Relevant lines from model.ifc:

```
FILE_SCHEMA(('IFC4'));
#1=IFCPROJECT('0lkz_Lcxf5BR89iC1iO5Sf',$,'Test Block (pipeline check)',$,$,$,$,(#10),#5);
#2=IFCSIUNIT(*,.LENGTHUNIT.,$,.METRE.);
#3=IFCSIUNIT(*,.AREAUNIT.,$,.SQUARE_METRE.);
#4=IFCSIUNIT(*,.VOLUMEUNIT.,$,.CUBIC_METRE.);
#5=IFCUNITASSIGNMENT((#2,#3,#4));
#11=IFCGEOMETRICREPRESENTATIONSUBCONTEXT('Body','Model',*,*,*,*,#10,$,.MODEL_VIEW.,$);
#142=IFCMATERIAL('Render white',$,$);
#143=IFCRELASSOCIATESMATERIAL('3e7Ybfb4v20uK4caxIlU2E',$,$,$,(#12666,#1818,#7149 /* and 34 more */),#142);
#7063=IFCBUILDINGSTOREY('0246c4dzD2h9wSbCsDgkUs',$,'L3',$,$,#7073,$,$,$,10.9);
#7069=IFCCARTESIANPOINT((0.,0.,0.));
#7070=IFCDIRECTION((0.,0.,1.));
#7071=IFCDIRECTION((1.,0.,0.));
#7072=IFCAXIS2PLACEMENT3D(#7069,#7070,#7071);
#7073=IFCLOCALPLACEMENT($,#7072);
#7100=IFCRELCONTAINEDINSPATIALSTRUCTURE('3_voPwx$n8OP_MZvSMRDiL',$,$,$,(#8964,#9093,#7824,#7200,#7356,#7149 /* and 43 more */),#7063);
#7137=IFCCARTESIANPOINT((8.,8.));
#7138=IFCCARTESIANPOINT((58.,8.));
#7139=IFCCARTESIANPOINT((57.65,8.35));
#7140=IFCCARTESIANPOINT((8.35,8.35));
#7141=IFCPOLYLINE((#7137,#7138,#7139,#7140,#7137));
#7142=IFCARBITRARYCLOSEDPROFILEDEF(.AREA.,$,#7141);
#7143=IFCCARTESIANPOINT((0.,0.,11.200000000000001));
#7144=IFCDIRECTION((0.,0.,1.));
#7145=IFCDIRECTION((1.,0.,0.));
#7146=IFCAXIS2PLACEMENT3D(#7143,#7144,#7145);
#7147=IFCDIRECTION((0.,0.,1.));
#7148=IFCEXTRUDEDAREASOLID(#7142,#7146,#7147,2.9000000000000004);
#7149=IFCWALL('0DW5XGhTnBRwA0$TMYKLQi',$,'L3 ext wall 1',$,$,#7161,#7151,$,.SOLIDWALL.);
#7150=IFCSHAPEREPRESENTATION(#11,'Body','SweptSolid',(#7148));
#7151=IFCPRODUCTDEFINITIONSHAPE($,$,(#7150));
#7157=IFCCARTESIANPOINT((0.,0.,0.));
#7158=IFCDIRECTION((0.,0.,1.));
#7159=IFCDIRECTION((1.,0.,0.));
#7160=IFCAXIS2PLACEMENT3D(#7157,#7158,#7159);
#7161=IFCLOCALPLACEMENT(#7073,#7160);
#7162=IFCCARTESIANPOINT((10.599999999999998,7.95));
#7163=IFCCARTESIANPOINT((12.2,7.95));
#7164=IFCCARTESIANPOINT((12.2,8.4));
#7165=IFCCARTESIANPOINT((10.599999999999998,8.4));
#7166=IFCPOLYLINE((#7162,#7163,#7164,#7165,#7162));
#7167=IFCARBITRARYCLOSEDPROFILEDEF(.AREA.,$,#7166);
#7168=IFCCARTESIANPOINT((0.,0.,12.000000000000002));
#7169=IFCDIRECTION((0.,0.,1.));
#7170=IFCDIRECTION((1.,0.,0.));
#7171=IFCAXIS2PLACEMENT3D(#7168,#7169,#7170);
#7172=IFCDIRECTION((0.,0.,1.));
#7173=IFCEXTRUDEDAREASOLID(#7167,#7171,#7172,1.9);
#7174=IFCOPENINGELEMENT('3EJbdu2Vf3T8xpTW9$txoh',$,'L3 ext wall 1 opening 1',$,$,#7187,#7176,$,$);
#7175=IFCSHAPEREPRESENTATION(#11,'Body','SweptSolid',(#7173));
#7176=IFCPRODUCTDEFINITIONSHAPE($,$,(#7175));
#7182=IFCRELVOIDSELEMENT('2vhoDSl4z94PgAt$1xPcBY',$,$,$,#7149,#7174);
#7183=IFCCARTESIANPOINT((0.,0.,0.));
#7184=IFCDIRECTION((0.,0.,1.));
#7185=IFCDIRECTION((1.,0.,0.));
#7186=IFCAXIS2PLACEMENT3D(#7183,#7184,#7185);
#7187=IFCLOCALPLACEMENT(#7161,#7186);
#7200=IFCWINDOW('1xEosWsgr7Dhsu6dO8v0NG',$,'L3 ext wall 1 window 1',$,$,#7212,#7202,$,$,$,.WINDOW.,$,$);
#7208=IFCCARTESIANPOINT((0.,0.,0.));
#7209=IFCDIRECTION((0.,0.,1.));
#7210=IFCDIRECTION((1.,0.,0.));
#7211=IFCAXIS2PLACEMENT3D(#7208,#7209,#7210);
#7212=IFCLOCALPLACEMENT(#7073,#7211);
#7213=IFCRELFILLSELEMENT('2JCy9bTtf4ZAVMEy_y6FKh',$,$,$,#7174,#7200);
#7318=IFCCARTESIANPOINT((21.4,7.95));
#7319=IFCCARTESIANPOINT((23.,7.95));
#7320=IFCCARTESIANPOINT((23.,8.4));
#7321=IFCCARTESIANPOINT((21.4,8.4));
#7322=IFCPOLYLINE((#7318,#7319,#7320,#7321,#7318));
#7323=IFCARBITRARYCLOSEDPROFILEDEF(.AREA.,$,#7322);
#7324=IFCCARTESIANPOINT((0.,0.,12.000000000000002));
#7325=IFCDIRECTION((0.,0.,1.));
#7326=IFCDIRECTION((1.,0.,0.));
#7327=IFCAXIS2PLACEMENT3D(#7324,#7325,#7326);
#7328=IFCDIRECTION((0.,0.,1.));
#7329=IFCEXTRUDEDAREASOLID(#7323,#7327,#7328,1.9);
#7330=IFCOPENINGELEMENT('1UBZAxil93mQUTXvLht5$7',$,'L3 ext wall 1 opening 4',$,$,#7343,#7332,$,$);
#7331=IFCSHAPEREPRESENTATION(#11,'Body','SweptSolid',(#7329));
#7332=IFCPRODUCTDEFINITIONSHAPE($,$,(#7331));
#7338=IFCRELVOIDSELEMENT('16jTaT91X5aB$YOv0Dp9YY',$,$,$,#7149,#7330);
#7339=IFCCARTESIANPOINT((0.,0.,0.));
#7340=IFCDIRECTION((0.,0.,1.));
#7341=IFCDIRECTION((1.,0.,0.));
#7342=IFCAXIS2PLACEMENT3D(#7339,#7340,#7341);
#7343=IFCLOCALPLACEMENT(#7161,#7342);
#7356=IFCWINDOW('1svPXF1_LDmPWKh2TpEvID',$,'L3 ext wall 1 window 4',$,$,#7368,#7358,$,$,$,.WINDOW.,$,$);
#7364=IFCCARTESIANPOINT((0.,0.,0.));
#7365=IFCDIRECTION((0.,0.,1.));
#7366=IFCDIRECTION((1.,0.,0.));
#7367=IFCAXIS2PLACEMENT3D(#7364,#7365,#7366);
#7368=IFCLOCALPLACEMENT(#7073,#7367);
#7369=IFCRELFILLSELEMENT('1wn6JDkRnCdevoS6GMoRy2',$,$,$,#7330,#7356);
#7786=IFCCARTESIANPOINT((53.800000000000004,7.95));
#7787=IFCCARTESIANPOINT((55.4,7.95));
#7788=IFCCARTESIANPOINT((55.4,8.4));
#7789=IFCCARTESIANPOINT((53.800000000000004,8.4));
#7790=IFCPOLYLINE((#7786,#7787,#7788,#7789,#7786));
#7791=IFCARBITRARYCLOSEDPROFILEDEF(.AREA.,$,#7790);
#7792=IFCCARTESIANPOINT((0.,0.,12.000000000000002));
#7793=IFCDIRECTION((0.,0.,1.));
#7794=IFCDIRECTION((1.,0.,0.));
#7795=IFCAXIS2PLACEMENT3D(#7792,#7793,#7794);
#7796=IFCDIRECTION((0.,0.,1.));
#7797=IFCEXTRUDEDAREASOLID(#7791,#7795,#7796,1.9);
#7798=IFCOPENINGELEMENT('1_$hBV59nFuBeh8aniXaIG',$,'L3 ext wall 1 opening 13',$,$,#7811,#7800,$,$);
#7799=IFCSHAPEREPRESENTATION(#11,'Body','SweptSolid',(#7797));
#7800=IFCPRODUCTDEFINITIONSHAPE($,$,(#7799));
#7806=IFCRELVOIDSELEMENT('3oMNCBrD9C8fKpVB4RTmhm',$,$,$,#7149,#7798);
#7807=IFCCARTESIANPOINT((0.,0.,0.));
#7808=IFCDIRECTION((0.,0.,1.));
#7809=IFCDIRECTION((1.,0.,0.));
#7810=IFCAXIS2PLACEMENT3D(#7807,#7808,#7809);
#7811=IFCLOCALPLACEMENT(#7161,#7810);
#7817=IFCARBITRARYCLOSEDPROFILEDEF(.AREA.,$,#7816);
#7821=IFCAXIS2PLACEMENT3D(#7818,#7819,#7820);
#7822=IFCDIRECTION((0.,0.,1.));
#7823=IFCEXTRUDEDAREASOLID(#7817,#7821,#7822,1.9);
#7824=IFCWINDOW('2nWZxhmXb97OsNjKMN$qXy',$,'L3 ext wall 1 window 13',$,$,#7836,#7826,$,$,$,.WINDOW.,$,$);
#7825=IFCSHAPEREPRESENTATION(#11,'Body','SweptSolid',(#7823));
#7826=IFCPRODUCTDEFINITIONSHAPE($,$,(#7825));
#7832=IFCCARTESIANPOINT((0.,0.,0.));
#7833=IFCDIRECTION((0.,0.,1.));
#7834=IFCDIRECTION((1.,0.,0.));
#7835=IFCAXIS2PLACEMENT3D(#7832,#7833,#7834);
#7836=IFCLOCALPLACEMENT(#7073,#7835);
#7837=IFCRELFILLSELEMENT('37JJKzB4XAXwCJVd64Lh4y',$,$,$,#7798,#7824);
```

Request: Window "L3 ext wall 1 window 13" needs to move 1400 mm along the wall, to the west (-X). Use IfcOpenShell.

```python
import ifcopenshell
import ifcopenshell.api.geometry
import ifcopenshell.util.placement
import ifcopenshell.util.unit

model = ifcopenshell.open("model.ifc")
unit_scale = ifcopenshell.util.unit.calculate_unit_scale(model)

window = model.by_id(7824)
opening = window.FillsVoids[0].RelatingOpeningElement
wall = opening.VoidsElements[0].RelatingBuildingElement

wall_matrix = ifcopenshell.util.placement.get_local_placement(wall.ObjectPlacement)
shift = wall_matrix[:3, 0] * -1.4 / unit_scale
before = ifcopenshell.util.placement.get_local_placement(window.ObjectPlacement)[:3, 3].copy()

# The window is not placed relative to its opening, so move both.
for product in (opening, window):
    matrix = ifcopenshell.util.placement.get_local_placement(product.ObjectPlacement)
    matrix[:3, 3] += shift
    ifcopenshell.api.geometry.edit_object_placement(model, product=product, matrix=matrix, is_si=False)

after = ifcopenshell.util.placement.get_local_placement(window.ObjectPlacement)[:3, 3]
print("window moved by", (after - before).round(3) + 0.0)

model.write("model_v2.ifc")
```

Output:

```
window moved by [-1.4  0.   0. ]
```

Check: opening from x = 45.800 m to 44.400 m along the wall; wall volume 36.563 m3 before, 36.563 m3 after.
